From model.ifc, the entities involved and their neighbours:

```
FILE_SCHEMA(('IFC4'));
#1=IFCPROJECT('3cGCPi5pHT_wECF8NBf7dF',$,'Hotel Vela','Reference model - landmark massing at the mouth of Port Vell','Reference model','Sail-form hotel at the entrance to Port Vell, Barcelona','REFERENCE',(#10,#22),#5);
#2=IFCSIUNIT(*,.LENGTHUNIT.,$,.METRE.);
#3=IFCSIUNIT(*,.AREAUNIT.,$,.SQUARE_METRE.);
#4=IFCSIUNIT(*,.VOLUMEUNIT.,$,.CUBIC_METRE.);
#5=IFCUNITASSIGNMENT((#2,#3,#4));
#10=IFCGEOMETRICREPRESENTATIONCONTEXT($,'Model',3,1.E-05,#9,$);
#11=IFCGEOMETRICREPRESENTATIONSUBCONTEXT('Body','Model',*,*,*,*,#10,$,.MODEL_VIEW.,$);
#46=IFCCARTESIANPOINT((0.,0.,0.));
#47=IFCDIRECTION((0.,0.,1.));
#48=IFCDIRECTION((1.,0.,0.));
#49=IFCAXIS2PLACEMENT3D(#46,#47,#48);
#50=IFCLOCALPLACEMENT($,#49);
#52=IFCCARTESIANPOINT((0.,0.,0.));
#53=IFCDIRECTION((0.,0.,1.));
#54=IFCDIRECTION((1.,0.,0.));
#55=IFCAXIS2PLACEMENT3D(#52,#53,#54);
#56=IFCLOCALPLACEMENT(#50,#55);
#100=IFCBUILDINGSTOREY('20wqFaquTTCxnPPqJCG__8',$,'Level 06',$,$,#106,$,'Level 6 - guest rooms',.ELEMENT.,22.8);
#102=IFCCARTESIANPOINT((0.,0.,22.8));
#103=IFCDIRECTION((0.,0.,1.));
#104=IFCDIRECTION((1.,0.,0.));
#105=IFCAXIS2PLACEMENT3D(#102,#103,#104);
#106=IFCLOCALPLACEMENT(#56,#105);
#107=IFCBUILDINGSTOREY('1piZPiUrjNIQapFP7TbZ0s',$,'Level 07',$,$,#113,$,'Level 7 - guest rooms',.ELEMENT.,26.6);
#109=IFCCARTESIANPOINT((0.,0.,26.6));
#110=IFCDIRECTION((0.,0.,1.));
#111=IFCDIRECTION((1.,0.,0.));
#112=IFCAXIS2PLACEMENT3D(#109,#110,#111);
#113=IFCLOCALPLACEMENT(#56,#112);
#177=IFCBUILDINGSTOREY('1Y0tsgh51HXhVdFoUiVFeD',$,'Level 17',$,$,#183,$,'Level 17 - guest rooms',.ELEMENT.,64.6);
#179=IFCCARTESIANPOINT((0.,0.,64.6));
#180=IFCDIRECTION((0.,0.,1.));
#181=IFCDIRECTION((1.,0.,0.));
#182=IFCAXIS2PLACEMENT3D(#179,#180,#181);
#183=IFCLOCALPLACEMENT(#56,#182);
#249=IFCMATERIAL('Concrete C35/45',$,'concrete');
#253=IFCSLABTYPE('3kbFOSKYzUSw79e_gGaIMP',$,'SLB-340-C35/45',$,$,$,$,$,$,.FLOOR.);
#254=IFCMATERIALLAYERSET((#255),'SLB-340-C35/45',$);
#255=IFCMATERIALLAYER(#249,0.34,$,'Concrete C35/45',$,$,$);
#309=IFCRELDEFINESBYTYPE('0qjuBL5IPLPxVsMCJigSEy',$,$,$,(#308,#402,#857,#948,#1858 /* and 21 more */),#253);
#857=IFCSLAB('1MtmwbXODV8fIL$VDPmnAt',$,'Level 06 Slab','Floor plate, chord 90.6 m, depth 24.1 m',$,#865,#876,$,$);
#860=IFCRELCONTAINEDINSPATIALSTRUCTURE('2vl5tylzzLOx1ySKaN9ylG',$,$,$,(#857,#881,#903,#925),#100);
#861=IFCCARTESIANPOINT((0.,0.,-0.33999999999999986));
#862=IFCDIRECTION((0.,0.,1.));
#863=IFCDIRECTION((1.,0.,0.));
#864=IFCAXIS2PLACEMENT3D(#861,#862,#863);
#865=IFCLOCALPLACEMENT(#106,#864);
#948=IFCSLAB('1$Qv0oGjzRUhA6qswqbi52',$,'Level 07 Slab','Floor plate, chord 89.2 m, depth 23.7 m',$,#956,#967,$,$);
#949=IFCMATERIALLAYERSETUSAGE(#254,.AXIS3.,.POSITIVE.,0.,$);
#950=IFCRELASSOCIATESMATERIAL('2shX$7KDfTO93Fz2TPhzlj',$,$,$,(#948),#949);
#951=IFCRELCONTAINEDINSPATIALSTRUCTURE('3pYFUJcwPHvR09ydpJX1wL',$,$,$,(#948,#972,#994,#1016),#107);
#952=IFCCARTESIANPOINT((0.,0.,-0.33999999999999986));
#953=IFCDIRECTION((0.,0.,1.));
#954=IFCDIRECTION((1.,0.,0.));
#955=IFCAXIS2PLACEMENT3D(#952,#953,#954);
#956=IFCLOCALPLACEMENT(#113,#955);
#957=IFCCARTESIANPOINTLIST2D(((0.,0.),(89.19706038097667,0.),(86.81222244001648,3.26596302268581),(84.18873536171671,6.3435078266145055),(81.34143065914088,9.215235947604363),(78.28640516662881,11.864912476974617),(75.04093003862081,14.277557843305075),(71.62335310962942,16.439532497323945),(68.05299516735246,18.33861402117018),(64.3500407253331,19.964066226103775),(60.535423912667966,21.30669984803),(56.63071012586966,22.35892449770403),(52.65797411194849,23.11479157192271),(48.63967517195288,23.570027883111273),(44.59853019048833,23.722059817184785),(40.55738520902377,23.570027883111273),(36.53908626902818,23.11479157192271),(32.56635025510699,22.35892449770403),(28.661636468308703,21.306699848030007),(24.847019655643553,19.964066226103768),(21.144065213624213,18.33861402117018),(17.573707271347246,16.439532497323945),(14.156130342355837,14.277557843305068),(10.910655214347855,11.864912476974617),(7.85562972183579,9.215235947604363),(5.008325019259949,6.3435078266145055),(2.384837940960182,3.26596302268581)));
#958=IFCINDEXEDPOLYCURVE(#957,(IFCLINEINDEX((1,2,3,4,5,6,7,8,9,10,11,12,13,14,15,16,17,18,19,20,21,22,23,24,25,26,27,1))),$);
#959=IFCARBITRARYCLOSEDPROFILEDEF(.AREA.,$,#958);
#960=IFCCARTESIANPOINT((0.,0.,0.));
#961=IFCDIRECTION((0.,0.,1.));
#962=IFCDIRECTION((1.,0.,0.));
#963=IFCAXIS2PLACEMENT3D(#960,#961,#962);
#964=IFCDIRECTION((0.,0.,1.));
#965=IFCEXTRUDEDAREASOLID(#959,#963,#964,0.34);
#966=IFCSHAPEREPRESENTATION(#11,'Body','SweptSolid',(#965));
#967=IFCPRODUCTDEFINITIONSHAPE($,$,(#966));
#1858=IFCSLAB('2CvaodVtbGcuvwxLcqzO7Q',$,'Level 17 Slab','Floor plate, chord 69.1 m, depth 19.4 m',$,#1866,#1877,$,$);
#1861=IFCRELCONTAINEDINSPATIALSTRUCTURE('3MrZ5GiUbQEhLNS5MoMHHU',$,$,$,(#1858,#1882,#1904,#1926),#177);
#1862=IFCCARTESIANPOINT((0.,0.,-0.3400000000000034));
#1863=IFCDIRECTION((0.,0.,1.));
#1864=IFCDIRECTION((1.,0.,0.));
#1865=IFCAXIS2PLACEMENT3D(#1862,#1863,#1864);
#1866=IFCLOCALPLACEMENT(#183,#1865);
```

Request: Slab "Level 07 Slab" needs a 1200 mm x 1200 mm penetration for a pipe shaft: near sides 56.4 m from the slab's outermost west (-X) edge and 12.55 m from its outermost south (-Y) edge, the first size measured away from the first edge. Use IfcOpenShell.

```python
import numpy as np
import ifcopenshell
import ifcopenshell.api.feature
import ifcopenshell.api.geometry
import ifcopenshell.api.root
import ifcopenshell.geom
import ifcopenshell.util.placement
import ifcopenshell.util.representation
import ifcopenshell.util.shape
import ifcopenshell.util.unit

model = ifcopenshell.open("model.ifc")
unit_scale = ifcopenshell.util.unit.calculate_unit_scale(model)
settings = ifcopenshell.geom.settings()


def volume(element):
    """Net volume in cubic metres, openings subtracted."""
    shape = ifcopenshell.geom.create_shape(settings, element)
    return ifcopenshell.util.shape.get_volume(shape.geometry)


slab = model.by_guid("1$Qv0oGjzRUhA6qswqbi52")
before = volume(slab)

# Extent in the slab's own axes, in metres. The edges named are its -X and -Y sides.
slab_shape = ifcopenshell.geom.create_shape(settings, slab)
vertices = ifcopenshell.util.shape.get_vertices(slab_shape.geometry)
x_min, y_min, bottom = vertices.min(axis=0)
top = vertices[:, 2].max()

opening = ifcopenshell.api.root.create_entity(model, ifc_class="IfcOpeningElement", name="Pipe shaft opening", predefined_type="OPENING")
context = ifcopenshell.util.representation.get_context(model, "Model", "Body", "MODEL_VIEW")
width, depth = 1.2, 1.2
outline = [(0.0, 0.0), (width, 0.0), (width, depth), (0.0, depth), (0.0, 0.0)]
# Overshoot both faces by 50 mm so the cut is clean.
shape = ifcopenshell.api.geometry.add_slab_representation(
    model, context=context, depth=top - bottom + 0.1, polyline=outline
)
ifcopenshell.api.geometry.assign_representation(model, product=opening, representation=shape)

matrix = ifcopenshell.util.placement.get_local_placement(slab.ObjectPlacement)
matrix[:, 3] = matrix @ np.append(np.array([x_min + 56.4, y_min + 12.55, bottom - 0.05]) / unit_scale, 1.0)
ifcopenshell.api.geometry.edit_object_placement(model, product=opening, matrix=matrix, is_si=False)
ifcopenshell.api.feature.add_feature(model, feature=opening, element=slab)

after = volume(slab)

print(f"slab volume {before:.3f} -> {after:.3f} m3")

model.write("model_v2.ifc")
```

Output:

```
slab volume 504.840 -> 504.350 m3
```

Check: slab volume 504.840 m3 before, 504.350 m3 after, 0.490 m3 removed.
